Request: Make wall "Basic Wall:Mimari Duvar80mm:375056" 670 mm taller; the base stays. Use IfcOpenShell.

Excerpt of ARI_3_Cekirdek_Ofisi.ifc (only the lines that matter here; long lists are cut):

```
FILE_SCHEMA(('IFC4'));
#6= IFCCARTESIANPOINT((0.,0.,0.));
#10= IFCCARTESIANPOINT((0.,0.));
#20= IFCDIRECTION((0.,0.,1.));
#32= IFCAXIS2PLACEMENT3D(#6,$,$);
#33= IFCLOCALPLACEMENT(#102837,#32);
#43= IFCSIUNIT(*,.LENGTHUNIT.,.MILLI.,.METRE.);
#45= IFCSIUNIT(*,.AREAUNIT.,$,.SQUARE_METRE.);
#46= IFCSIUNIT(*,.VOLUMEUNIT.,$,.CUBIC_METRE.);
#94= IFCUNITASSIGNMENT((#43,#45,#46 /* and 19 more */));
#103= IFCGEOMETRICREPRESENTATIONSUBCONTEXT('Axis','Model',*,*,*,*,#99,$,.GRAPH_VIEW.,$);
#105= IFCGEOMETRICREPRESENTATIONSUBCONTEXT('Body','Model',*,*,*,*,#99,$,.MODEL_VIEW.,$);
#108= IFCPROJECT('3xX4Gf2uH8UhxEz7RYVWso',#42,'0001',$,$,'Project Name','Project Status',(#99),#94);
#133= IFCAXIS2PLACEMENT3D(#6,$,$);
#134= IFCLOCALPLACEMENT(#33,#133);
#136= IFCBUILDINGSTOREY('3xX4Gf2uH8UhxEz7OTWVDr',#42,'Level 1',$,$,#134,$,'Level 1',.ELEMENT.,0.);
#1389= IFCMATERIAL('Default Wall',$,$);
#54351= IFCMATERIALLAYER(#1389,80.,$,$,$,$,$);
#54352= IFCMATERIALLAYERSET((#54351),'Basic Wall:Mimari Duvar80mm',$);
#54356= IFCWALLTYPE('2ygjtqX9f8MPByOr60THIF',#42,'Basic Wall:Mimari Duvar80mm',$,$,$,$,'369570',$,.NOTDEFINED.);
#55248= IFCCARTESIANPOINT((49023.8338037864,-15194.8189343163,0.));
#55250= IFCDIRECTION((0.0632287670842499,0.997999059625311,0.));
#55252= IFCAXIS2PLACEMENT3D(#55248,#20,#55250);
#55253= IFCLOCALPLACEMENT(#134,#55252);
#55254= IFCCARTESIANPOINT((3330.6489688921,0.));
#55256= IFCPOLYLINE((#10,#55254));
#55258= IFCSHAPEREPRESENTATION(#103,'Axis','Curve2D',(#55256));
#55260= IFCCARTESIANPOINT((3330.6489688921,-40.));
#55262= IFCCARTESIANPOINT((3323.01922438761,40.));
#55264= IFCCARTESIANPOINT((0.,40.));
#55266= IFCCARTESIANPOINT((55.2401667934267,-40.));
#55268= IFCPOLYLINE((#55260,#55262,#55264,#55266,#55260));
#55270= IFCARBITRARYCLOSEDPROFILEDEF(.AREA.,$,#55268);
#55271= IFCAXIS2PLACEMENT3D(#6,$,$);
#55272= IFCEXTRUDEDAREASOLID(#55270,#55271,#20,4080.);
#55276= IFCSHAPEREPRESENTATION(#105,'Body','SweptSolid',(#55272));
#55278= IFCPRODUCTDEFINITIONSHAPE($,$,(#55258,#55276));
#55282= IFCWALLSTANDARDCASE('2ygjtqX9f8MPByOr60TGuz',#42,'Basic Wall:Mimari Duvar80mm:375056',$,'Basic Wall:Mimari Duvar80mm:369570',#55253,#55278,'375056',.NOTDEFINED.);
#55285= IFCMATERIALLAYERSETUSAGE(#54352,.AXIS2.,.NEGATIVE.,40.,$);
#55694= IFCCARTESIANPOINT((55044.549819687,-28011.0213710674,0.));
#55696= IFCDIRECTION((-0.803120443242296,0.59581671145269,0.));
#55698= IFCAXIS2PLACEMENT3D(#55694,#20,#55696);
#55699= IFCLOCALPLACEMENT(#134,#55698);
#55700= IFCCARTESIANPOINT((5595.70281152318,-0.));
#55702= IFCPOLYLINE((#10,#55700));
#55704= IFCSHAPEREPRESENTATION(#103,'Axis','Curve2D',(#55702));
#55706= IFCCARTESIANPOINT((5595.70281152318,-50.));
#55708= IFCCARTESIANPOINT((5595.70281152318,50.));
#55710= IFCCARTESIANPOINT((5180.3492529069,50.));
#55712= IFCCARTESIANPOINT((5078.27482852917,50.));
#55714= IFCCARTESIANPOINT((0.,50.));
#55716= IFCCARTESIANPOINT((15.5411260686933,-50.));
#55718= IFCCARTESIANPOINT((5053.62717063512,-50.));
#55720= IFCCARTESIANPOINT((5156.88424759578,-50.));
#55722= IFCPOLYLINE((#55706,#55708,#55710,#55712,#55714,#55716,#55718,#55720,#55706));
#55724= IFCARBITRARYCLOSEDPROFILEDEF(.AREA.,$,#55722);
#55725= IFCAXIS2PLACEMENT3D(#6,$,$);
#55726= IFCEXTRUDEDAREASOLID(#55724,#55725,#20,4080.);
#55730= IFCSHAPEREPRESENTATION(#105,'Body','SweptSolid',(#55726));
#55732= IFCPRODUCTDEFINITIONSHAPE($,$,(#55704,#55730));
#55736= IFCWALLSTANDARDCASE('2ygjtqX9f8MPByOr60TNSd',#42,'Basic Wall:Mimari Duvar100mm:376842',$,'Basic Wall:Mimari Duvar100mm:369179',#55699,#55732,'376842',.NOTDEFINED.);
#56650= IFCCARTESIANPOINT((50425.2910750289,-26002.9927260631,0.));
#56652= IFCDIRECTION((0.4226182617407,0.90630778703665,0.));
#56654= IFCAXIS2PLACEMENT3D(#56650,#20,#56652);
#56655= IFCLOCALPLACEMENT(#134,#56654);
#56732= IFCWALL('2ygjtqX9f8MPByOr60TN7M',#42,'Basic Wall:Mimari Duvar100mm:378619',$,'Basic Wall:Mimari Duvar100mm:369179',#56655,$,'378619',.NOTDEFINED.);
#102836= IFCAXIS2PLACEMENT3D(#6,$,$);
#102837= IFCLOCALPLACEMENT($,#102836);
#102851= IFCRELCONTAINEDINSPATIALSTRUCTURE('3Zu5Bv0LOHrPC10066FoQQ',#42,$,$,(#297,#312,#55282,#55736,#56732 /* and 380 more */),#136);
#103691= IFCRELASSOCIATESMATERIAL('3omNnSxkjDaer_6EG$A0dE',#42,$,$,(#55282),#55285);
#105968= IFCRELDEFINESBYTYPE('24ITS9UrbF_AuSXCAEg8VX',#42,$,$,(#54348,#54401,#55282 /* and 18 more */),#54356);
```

```python
import ifcopenshell
import ifcopenshell.geom
import ifcopenshell.util.representation
import ifcopenshell.util.shape
import ifcopenshell.util.unit

model = ifcopenshell.open("ARI_3_Cekirdek_Ofisi.ifc")
unit_scale = ifcopenshell.util.unit.calculate_unit_scale(model)
settings = ifcopenshell.geom.settings()


def volume(element):
    """Net volume in cubic metres, openings subtracted."""
    shape = ifcopenshell.geom.create_shape(settings, element)
    return ifcopenshell.util.shape.get_volume(shape.geometry)


wall = model.by_id(55282)
before = volume(wall)

body = ifcopenshell.util.representation.get_representation(wall, "Model", "Body")
solid = body.Items[0]
old_height = solid.Depth
solid.Depth += 0.67 / unit_scale
after = volume(wall)

print(f"height {old_height:g} -> {solid.Depth:g}, volume {before:.3f} -> {after:.3f} m3")

model.write("ARI_3_Cekirdek_Ofisi_updated.ifc")
```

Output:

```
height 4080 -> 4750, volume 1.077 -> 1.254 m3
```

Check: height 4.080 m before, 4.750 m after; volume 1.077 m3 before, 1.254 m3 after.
